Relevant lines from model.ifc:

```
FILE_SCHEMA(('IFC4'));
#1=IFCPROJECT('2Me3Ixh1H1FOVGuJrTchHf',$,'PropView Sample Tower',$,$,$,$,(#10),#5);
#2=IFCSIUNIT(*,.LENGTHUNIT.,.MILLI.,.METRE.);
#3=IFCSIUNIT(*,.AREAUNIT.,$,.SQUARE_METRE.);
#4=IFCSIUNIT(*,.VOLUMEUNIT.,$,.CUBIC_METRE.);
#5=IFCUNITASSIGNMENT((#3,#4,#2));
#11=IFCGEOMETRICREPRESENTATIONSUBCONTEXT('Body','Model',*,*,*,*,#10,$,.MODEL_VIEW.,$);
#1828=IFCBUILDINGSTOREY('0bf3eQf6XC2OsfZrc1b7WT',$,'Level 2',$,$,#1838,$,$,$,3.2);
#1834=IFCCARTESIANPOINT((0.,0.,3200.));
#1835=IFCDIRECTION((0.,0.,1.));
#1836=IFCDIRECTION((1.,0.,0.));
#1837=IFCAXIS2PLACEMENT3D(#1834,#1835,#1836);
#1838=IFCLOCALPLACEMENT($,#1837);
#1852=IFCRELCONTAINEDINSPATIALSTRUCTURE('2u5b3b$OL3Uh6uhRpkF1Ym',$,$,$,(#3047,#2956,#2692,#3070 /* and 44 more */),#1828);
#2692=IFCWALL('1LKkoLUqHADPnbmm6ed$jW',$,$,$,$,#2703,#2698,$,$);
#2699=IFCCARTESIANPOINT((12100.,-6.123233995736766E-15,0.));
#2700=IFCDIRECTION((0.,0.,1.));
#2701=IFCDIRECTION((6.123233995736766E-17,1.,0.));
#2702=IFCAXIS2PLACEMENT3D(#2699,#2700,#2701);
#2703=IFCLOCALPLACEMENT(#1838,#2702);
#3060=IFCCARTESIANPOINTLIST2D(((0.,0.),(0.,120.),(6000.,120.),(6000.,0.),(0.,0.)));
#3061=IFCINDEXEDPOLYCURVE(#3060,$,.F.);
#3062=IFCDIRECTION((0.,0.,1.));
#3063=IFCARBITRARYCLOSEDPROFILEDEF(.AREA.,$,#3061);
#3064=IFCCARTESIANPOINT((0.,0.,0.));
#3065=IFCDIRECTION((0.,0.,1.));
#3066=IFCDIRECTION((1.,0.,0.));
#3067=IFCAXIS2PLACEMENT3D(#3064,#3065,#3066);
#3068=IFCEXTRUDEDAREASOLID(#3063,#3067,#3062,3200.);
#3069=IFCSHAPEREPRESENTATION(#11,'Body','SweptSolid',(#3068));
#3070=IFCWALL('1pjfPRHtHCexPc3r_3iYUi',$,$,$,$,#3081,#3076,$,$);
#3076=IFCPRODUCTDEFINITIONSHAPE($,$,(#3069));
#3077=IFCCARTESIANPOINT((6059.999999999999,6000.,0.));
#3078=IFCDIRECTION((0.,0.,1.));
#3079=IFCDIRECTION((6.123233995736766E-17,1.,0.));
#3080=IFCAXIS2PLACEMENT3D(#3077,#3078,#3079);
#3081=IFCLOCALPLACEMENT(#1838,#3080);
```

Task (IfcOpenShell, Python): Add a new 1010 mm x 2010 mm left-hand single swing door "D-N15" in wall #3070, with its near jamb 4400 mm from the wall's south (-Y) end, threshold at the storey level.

```python
import numpy as np
import ifcopenshell
import ifcopenshell.api.feature
import ifcopenshell.api.geometry
import ifcopenshell.api.root
import ifcopenshell.api.spatial
import ifcopenshell.geom
import ifcopenshell.util.element
import ifcopenshell.util.placement
import ifcopenshell.util.representation
import ifcopenshell.util.shape
import ifcopenshell.util.unit

model = ifcopenshell.open("model.ifc")
unit_scale = ifcopenshell.util.unit.calculate_unit_scale(model)
settings = ifcopenshell.geom.settings()


def volume(element):
    """Net volume in cubic metres, openings subtracted."""
    shape = ifcopenshell.geom.create_shape(settings, element)
    return ifcopenshell.util.shape.get_volume(shape.geometry)


wall = model.by_id(3070)
storey = ifcopenshell.util.element.get_container(wall, ifc_class="IfcBuildingStorey")
context = ifcopenshell.util.representation.get_context(model, "Model", "Body", "MODEL_VIEW")
before = volume(wall)

width, height, from_end, sill = 1.01, 2.01, 4.4, 0.0  # metres

# The wall runs along its own X axis, and the end named is its -X end.
wall_shape = ifcopenshell.geom.create_shape(settings, wall)
x, y, z = ifcopenshell.util.shape.get_vertices(wall_shape.geometry).T
start = x.min() + from_end
face, thickness = float(y.min()), float(y.max() - y.min())
wall_matrix = ifcopenshell.util.placement.get_local_placement(wall.ObjectPlacement)
level = ifcopenshell.util.placement.get_local_placement(storey.ObjectPlacement)[2, 3]


def in_wall(x, y):
    """Placement at x, y metres in the wall's axes, at sill height."""
    matrix = wall_matrix.copy()
    matrix[:, 3] = wall_matrix @ np.array([x / unit_scale, y / unit_scale, 0.0, 1.0])
    matrix[2, 3] = level + sill / unit_scale
    return matrix


# Opening: a box that overshoots both wall faces by 50 mm.
opening = ifcopenshell.api.root.create_entity(model, ifc_class="IfcOpeningElement", predefined_type="OPENING")
box = ifcopenshell.api.geometry.add_wall_representation(
    model, context=context, length=width, height=height, thickness=thickness + 0.1
)
ifcopenshell.api.geometry.assign_representation(model, product=opening, representation=box)
ifcopenshell.api.geometry.edit_object_placement(model, product=opening, matrix=in_wall(start, face - 0.05), is_si=False)
ifcopenshell.api.feature.add_feature(model, feature=opening, element=wall)

door = ifcopenshell.api.root.create_entity(model, ifc_class="IfcDoor", name="D-N15", predefined_type="DOOR")
door.OverallWidth, door.OverallHeight = width / unit_scale, height / unit_scale
door.OperationType = "SINGLE_SWING_LEFT"
body = ifcopenshell.api.geometry.add_door_representation(
    model,
    context=context,
    overall_width=door.OverallWidth,
    overall_height=door.OverallHeight,
    operation_type="SINGLE_SWING_LEFT",
    lining_properties={"LiningDepth": thickness / unit_scale, "ThresholdDepth": thickness / unit_scale},
)
ifcopenshell.api.geometry.assign_representation(model, product=door, representation=body)
ifcopenshell.api.spatial.assign_container(model, products=[door], relating_structure=storey)
ifcopenshell.api.feature.add_filling(model, opening=opening, element=door)

# The lining spans the wall, so the door starts at the wall face.
ifcopenshell.api.geometry.edit_object_placement(model, product=door, matrix=in_wall(start, face), is_si=False)

after = volume(wall)

print(f"wall volume {before:.3f} -> {after:.3f} m3")

model.write("model-out.ifc")
```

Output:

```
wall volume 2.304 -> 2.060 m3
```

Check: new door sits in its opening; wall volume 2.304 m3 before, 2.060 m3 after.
